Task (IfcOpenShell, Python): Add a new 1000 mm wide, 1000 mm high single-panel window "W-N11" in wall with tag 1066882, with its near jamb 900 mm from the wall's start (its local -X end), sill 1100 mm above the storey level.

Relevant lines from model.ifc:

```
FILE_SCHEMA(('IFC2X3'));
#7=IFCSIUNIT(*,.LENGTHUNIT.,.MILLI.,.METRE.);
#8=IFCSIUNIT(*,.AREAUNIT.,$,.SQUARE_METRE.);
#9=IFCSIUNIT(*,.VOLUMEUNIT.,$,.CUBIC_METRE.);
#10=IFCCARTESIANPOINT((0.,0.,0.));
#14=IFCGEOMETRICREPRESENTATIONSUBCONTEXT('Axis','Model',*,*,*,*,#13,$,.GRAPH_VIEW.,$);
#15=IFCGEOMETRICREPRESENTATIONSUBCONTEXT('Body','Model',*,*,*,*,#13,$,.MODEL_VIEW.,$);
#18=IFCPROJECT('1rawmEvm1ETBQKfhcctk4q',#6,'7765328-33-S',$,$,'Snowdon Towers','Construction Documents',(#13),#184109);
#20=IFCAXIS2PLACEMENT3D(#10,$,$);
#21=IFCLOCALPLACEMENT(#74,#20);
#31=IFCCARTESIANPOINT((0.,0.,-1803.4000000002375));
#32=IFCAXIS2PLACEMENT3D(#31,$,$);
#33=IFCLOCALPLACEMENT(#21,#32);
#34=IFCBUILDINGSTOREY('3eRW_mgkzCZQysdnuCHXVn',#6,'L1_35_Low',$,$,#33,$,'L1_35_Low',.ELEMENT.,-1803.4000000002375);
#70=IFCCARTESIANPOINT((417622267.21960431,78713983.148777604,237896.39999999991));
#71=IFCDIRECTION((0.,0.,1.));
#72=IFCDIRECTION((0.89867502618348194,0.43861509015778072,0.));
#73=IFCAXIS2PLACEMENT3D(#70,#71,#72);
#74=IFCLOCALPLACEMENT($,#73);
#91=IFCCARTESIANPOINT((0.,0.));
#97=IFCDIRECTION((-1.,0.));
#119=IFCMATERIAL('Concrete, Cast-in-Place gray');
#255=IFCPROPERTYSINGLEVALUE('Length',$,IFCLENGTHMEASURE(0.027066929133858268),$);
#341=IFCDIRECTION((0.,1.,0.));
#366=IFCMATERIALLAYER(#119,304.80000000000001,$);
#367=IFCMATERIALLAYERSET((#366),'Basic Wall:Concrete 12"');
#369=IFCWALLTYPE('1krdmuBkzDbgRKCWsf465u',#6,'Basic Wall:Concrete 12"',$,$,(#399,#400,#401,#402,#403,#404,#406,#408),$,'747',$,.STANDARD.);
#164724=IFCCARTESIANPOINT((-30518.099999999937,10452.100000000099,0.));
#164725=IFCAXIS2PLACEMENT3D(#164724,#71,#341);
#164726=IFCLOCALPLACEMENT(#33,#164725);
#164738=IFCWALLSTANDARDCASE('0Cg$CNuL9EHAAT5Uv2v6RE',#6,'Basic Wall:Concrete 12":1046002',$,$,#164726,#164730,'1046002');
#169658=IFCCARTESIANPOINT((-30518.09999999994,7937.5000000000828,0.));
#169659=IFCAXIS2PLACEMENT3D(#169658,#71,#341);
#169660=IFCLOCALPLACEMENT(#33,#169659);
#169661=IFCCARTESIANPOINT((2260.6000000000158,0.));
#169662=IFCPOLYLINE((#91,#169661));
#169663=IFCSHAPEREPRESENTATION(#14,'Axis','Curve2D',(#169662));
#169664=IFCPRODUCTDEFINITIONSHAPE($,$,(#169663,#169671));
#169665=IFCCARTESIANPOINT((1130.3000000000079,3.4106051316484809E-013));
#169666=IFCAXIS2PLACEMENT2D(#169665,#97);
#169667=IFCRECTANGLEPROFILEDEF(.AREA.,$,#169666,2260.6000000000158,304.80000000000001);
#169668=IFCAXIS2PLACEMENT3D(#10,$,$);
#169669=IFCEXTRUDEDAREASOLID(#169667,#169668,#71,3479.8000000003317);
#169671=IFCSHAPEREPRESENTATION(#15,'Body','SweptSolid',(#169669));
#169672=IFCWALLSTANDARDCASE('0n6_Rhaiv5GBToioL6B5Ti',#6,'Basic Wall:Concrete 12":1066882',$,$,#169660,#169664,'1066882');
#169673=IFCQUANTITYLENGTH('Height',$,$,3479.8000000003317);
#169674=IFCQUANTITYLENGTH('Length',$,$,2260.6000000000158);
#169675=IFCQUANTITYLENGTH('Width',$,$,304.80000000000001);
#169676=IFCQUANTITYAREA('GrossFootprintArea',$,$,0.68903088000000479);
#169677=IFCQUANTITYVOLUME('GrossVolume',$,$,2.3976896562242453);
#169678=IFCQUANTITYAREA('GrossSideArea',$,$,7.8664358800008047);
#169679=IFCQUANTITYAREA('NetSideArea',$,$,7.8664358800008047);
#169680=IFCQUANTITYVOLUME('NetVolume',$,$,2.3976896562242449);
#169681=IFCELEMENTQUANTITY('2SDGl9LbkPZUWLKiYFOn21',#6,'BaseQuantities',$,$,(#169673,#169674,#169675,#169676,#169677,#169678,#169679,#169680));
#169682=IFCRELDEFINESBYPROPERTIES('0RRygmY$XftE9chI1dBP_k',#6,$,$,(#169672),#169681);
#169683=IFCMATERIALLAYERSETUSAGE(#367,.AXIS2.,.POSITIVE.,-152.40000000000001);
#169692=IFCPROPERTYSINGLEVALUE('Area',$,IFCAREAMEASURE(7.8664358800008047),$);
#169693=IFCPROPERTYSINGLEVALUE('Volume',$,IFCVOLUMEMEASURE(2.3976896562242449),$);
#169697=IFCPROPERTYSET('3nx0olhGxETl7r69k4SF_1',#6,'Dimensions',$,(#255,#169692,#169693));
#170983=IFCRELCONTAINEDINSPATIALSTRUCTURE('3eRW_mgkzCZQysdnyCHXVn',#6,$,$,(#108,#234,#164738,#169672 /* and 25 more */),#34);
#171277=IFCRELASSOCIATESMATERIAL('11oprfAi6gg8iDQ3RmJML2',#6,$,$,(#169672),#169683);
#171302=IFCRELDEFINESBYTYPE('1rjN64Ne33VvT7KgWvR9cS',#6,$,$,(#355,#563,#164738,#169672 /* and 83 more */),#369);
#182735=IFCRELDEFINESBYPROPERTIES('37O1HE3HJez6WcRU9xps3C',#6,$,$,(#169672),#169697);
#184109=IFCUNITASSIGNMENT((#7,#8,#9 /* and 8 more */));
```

```python
import numpy as np
import ifcopenshell
import ifcopenshell.api.feature
import ifcopenshell.api.geometry
import ifcopenshell.api.pset
import ifcopenshell.api.root
import ifcopenshell.api.spatial
import ifcopenshell.api.type
import ifcopenshell.geom
import ifcopenshell.util.element
import ifcopenshell.util.placement
import ifcopenshell.util.representation
import ifcopenshell.util.shape
import ifcopenshell.util.unit

model = ifcopenshell.open("model.ifc")
unit_scale = ifcopenshell.util.unit.calculate_unit_scale(model)
area_scale = ifcopenshell.util.unit.calculate_unit_scale(model, "AREAUNIT")
volume_scale = ifcopenshell.util.unit.calculate_unit_scale(model, "VOLUMEUNIT")
settings = ifcopenshell.geom.settings()


def volume(element):
    """Net volume in cubic metres, openings subtracted."""
    shape = ifcopenshell.geom.create_shape(settings, element)
    return ifcopenshell.util.shape.get_volume(shape.geometry)


wall = model.by_guid("0n6_Rhaiv5GBToioL6B5Ti")
storey = ifcopenshell.util.element.get_container(wall, ifc_class="IfcBuildingStorey")
context = ifcopenshell.util.representation.get_context(model, "Model", "Body", "MODEL_VIEW")
before = volume(wall)

width, height, from_end, sill = 1, 1, 0.9, 1.1  # metres

# The wall runs along its own X axis, and the end named is its -X end.
wall_shape = ifcopenshell.geom.create_shape(settings, wall)
x, y, z = ifcopenshell.util.shape.get_vertices(wall_shape.geometry).T
start = x.min() + from_end
face, thickness = float(y.min()), float(y.max() - y.min())
wall_matrix = ifcopenshell.util.placement.get_local_placement(wall.ObjectPlacement)
level = ifcopenshell.util.placement.get_local_placement(storey.ObjectPlacement)[2, 3]


def in_wall(x, y):
    """Placement at x, y metres in the wall's axes, at sill height."""
    matrix = wall_matrix.copy()
    matrix[:, 3] = wall_matrix @ np.array([x / unit_scale, y / unit_scale, 0.0, 1.0])
    matrix[2, 3] = level + sill / unit_scale
    return matrix


# Opening: a box that overshoots both wall faces by 50 mm.
opening = ifcopenshell.api.root.create_entity(model, ifc_class="IfcOpeningElement")
box = ifcopenshell.api.geometry.add_wall_representation(
    model, context=context, length=width, height=height, thickness=thickness + 0.1
)
ifcopenshell.api.geometry.assign_representation(model, product=opening, representation=box)
ifcopenshell.api.geometry.edit_object_placement(model, product=opening, matrix=in_wall(start, face - 0.05), is_si=False)
ifcopenshell.api.feature.add_feature(model, feature=opening, element=wall)

window = ifcopenshell.api.root.create_entity(model, ifc_class="IfcWindow", name="W-N11")
window.OverallWidth, window.OverallHeight = width / unit_scale, height / unit_scale
body = ifcopenshell.api.geometry.add_window_representation(
    model,
    context=context,
    overall_width=window.OverallWidth,
    overall_height=window.OverallHeight,
    partition_type="SINGLE_PANEL",
)
ifcopenshell.api.geometry.assign_representation(model, product=window, representation=body)
ifcopenshell.api.spatial.assign_container(model, products=[window], relating_structure=storey)
fills = ifcopenshell.api.feature.add_filling(model, opening=opening, element=window)
fills.OwnerHistory = window.OwnerHistory  # required in IFC2X3

# IFC2X3 keeps the operation on the window style.
style = ifcopenshell.api.root.create_entity(model, ifc_class="IfcWindowStyle", name="W-N11")
style.OperationType, style.ConstructionType = "SINGLE_PANEL", "NOTDEFINED"
style.ParameterTakesPrecedence = style.Sizeable = False
ifcopenshell.api.type.assign_type(model, related_objects=[window], relating_type=style)

# Centre the window in the wall's thickness.
ifcopenshell.api.geometry.edit_object_placement(model, product=window, matrix=in_wall(start, face), is_si=False)
window_shape = ifcopenshell.geom.create_shape(settings, window)
depth = ifcopenshell.util.shape.get_vertices(window_shape.geometry)[:, 1]
offset = face + thickness / 2 - (depth.min() + depth.max()) / 2
ifcopenshell.api.geometry.edit_object_placement(model, product=window, matrix=in_wall(start, offset), is_si=False)

after = volume(wall)

# Update the wall's stored quantities.
qto = model.by_id(ifcopenshell.util.element.get_pset(wall, "BaseQuantities", should_inherit=False)["id"])
ifcopenshell.api.pset.edit_qto(model, qto=qto, properties={
    "NetSideArea": after / thickness / area_scale,
    "NetVolume": after / volume_scale,
})
pset = model.by_id(ifcopenshell.util.element.get_pset(wall, "Dimensions", should_inherit=False)["id"])
ifcopenshell.api.pset.edit_pset(model, pset=pset, properties={
    "Area": model.create_entity("IfcAreaMeasure", after / thickness / area_scale),
    "Volume": model.create_entity("IfcVolumeMeasure", after / volume_scale),
})

print(f"wall volume {before:.3f} -> {after:.3f} m3")

model.write("model_rev.ifc")
```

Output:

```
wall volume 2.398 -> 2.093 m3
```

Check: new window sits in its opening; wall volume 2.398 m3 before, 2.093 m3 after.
